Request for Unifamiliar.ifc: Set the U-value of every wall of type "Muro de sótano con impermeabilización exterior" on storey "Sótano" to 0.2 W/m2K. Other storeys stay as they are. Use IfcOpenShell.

First a look at what the model holds.

```python
import ifcopenshell
import ifcopenshell.util.element

model = ifcopenshell.open("Unifamiliar.ifc")
print(model.schema)
storey = next(s for s in model.by_type("IfcBuildingStorey") if s.Name == "Sótano")
walls = [e for e in ifcopenshell.util.element.get_decomposition(storey) if e.is_a("IfcWall")]
seen = {}
for e in walls:
    element_type = ifcopenshell.util.element.get_type(e)
    key = (element_type.Name if element_type != e and element_type else None, ifcopenshell.util.element.get_pset(e, "Pset_WallCommon", "ThermalTransmittance"))
    seen[key] = seen.get(key, 0) + 1
for (name, value), count in sorted(seen.items(), key=str):
    print(count, "x", name, "|", value)
```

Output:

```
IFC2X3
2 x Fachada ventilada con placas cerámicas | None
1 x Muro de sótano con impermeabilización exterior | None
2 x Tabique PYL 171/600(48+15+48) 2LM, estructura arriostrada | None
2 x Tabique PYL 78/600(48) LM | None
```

```python
import ifcopenshell
import ifcopenshell.api.pset
import ifcopenshell.util.element

model = ifcopenshell.open("Unifamiliar.ifc")

storey = next(s for s in model.by_type("IfcBuildingStorey") if s.Name == "Sótano")
walls = [e for e in ifcopenshell.util.element.get_decomposition(storey) if e.is_a("IfcWall")]

count = 0
for e in walls:
    element_type = ifcopenshell.util.element.get_type(e)
    if element_type in (None, e) or element_type.Name != "Muro de sótano con impermeabilización exterior":
        continue
    # add_pset returns the element's existing set when there is one.
    pset = ifcopenshell.api.pset.add_pset(model, product=e, name="Pset_WallCommon")
    ifcopenshell.api.pset.edit_pset(model, pset=pset, properties={"ThermalTransmittance": 0.2})
    count += 1

print(count, "walls updated")

model.write("Unifamiliar_v2.ifc")
```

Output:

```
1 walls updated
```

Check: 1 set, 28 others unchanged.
